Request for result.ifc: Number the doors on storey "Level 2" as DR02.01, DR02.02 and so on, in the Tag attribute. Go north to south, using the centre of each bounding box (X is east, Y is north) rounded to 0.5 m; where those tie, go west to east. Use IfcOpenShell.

First a look at what the model holds.

```python
import ifcopenshell
import ifcopenshell.util.element
import ifcopenshell.util.placement

model = ifcopenshell.open("result.ifc")
print(model.schema)
storey = next(s for s in model.by_type("IfcBuildingStorey") if s.Name == "Level 2")
doors = [e for e in ifcopenshell.util.element.get_decomposition(storey) if e.is_a("IfcDoor")]
for e in sorted(doors, key=lambda e: e.id()):
    origin = ifcopenshell.util.placement.get_local_placement(e.ObjectPlacement)[:3, 3]
    print(e.id(), e.Tag, e.Name, origin.round(2) + 0.0, sep=" | ")
```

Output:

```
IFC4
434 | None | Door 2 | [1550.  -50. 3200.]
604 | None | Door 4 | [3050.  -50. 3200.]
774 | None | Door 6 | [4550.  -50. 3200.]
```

```python
import ifcopenshell
import ifcopenshell.geom
import ifcopenshell.util.element
import ifcopenshell.util.shape

model = ifcopenshell.open("result.ifc")
settings = ifcopenshell.geom.settings()
settings.set("use-world-coords", True)


def centre(element):
    shape = ifcopenshell.geom.create_shape(settings, element)
    return ifcopenshell.util.shape.get_bbox_centroid(shape.geometry)


storey = next(s for s in model.by_type("IfcBuildingStorey") if s.Name == "Level 2")
doors = [e for e in ifcopenshell.util.element.get_decomposition(storey) if e.is_a("IfcDoor")]

# Insertion points can sit at a corner or the storey origin, so sort by the geometry (in metres).
centres = {e: centre(e) for e in doors}
doors.sort(key=lambda e: (-round(centres[e][1] / 0.5), centres[e][0]))

for i, e in enumerate(doors, start=1):
    number = f"DR02.{i:02d}"
    e.Tag = number
    print(e.id(), number)

model.write("result_rev.ifc")
```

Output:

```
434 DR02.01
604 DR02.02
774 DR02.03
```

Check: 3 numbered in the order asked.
